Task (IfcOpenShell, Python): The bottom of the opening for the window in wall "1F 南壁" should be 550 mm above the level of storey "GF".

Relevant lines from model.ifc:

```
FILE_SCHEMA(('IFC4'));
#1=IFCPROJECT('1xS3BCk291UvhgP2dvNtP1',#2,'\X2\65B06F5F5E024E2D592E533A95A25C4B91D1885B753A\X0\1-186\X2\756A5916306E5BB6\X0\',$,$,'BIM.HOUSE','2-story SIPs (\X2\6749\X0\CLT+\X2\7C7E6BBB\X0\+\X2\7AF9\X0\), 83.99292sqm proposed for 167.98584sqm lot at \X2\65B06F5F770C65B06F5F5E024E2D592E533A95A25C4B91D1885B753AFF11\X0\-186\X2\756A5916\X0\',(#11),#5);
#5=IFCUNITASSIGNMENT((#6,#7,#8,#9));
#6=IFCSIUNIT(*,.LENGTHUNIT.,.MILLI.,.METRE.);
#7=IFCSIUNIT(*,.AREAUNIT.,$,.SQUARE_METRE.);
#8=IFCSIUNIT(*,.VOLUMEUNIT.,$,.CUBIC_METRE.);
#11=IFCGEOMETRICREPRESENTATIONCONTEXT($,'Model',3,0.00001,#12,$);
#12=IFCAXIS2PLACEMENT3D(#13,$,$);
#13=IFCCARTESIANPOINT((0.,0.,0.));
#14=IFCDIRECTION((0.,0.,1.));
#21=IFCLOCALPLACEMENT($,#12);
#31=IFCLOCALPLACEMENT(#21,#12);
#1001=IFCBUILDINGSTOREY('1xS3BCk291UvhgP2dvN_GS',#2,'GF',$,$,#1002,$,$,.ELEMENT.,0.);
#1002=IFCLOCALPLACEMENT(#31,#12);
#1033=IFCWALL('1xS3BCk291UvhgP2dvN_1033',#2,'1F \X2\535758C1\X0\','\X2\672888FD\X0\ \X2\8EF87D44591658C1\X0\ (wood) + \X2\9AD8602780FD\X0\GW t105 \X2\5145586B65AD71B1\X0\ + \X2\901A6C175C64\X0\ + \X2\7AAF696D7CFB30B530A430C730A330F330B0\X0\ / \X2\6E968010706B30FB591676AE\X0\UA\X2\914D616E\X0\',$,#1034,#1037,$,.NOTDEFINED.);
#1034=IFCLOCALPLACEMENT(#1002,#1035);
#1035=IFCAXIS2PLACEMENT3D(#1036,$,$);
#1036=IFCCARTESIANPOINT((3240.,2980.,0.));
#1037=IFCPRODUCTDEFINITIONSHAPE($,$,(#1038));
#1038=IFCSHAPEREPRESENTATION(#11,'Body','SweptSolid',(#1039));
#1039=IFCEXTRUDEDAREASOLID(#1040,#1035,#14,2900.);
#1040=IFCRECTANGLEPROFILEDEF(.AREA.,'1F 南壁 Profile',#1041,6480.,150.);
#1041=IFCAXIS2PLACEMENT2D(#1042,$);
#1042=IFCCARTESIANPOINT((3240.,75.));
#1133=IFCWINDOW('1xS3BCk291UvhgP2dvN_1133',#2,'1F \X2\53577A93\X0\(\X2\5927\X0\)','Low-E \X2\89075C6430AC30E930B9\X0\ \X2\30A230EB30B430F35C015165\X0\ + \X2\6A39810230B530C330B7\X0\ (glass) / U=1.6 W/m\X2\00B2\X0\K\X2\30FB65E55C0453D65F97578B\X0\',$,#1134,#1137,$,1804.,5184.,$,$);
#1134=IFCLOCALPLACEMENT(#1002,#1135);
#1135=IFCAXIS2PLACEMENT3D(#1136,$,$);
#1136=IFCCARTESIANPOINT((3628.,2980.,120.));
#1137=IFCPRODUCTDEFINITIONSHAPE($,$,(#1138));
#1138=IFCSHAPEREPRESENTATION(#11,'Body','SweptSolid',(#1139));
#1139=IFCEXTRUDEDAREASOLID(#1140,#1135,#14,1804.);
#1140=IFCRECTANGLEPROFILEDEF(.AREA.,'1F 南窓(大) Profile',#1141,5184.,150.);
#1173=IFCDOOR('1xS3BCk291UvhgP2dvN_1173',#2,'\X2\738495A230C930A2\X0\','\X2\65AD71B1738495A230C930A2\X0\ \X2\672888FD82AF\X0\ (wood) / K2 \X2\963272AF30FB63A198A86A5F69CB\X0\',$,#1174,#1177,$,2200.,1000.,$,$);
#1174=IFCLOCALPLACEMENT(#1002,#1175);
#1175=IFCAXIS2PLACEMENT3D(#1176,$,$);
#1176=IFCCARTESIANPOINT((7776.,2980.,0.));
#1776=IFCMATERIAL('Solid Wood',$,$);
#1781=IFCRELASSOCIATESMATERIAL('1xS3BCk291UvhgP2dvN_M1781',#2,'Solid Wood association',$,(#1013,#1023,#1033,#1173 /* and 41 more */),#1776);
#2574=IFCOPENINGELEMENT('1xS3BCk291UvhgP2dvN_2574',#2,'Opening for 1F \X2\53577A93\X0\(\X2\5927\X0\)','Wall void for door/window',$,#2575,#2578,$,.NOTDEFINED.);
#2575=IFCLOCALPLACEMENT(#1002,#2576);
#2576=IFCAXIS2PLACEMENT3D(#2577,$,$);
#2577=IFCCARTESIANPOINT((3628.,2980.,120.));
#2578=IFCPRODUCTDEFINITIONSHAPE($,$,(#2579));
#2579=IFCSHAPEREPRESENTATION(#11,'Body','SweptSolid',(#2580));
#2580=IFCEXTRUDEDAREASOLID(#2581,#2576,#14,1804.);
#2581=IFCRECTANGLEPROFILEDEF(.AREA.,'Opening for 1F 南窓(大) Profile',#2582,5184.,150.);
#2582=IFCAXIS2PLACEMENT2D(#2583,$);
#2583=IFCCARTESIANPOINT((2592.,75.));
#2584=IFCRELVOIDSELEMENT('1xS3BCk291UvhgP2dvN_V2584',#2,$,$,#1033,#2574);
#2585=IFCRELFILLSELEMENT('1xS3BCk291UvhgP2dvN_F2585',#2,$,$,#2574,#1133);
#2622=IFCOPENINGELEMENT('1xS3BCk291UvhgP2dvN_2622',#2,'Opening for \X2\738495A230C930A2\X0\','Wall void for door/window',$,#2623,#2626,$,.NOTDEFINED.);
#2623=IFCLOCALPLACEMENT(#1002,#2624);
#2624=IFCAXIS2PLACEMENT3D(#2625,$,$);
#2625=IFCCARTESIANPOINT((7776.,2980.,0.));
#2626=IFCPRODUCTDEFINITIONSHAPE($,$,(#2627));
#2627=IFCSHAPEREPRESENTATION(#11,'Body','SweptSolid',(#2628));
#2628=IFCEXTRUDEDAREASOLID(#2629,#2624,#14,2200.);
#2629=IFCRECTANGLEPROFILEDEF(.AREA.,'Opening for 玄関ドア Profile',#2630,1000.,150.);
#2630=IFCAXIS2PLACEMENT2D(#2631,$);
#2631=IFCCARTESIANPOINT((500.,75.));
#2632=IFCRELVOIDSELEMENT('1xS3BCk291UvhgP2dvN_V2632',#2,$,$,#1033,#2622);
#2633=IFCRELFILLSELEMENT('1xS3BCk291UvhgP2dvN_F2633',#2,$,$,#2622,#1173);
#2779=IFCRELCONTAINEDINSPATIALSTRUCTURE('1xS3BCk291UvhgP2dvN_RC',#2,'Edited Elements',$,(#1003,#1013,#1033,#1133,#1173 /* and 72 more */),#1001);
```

```python
import numpy as np
import ifcopenshell
import ifcopenshell.api.geometry
import ifcopenshell.geom
import ifcopenshell.util.element
import ifcopenshell.util.placement
import ifcopenshell.util.shape
import ifcopenshell.util.unit

model = ifcopenshell.open("model.ifc")
unit_scale = ifcopenshell.util.unit.calculate_unit_scale(model)

window = model.by_guid("1xS3BCk291UvhgP2dvN_1133")
opening = window.FillsVoids[0].RelatingOpeningElement
storey = ifcopenshell.util.element.get_container(window, ifc_class="IfcBuildingStorey")
level = ifcopenshell.util.placement.get_local_placement(storey.ObjectPlacement)[2, 3]

# The opening's origin need not be at the sill, so measure its lowest point.
shape = ifcopenshell.geom.create_shape(ifcopenshell.geom.settings(), opening)
bottom = ifcopenshell.util.shape.get_shape_bottom_elevation(shape, shape.geometry) / unit_scale
dz = level + 550.0 - bottom

shift = np.array([0.0, 0.0, dz])
# The window is not placed relative to its opening, so move both.
for product in (opening, window):
    matrix = ifcopenshell.util.placement.get_local_placement(product.ObjectPlacement)
    matrix[:3, 3] += shift
    ifcopenshell.api.geometry.edit_object_placement(model, product=product, matrix=matrix, is_si=False)

print(f"moved by {dz * unit_scale:+.3f} m")

model.write("model_updated.ifc")
```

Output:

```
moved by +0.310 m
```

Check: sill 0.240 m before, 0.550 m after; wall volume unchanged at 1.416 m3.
